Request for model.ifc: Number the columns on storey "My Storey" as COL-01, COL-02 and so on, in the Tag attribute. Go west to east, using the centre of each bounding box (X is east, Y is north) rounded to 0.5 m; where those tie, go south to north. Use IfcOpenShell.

First a look at what the model holds.

```python
import ifcopenshell
import ifcopenshell.util.element
import ifcopenshell.util.placement

model = ifcopenshell.open("model.ifc")
print(model.schema)
storey = next(s for s in model.by_type("IfcBuildingStorey") if s.Name == "My Storey")
columns = [e for e in ifcopenshell.util.element.get_decomposition(storey) if e.is_a("IfcColumn")]
for e in sorted(columns, key=lambda e: e.id()):
    origin = ifcopenshell.util.placement.get_local_placement(e.ObjectPlacement)[:3, 3]
    print(e.id(), e.Tag, e.Name, origin.round(2) + 0.0, sep=" | ")
```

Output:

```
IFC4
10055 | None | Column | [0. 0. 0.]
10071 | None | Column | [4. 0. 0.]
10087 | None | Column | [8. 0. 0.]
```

```python
import ifcopenshell
import ifcopenshell.geom
import ifcopenshell.util.element
import ifcopenshell.util.shape

model = ifcopenshell.open("model.ifc")
settings = ifcopenshell.geom.settings()
settings.set("use-world-coords", True)


def centre(element):
    shape = ifcopenshell.geom.create_shape(settings, element)
    return ifcopenshell.util.shape.get_bbox_centroid(shape.geometry)


storey = next(s for s in model.by_type("IfcBuildingStorey") if s.Name == "My Storey")
columns = [e for e in ifcopenshell.util.element.get_decomposition(storey) if e.is_a("IfcColumn")]

# Insertion points can sit at a corner or the storey origin, so sort by the geometry (in metres).
centres = {e: centre(e) for e in columns}
columns.sort(key=lambda e: (round(centres[e][0] / 0.5), centres[e][1]))

for i, e in enumerate(columns, start=1):
    number = f"COL-{i:02d}"
    e.Tag = number
    print(e.id(), number)

model.write("model-out.ifc")
```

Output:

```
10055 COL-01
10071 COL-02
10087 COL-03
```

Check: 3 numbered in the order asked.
